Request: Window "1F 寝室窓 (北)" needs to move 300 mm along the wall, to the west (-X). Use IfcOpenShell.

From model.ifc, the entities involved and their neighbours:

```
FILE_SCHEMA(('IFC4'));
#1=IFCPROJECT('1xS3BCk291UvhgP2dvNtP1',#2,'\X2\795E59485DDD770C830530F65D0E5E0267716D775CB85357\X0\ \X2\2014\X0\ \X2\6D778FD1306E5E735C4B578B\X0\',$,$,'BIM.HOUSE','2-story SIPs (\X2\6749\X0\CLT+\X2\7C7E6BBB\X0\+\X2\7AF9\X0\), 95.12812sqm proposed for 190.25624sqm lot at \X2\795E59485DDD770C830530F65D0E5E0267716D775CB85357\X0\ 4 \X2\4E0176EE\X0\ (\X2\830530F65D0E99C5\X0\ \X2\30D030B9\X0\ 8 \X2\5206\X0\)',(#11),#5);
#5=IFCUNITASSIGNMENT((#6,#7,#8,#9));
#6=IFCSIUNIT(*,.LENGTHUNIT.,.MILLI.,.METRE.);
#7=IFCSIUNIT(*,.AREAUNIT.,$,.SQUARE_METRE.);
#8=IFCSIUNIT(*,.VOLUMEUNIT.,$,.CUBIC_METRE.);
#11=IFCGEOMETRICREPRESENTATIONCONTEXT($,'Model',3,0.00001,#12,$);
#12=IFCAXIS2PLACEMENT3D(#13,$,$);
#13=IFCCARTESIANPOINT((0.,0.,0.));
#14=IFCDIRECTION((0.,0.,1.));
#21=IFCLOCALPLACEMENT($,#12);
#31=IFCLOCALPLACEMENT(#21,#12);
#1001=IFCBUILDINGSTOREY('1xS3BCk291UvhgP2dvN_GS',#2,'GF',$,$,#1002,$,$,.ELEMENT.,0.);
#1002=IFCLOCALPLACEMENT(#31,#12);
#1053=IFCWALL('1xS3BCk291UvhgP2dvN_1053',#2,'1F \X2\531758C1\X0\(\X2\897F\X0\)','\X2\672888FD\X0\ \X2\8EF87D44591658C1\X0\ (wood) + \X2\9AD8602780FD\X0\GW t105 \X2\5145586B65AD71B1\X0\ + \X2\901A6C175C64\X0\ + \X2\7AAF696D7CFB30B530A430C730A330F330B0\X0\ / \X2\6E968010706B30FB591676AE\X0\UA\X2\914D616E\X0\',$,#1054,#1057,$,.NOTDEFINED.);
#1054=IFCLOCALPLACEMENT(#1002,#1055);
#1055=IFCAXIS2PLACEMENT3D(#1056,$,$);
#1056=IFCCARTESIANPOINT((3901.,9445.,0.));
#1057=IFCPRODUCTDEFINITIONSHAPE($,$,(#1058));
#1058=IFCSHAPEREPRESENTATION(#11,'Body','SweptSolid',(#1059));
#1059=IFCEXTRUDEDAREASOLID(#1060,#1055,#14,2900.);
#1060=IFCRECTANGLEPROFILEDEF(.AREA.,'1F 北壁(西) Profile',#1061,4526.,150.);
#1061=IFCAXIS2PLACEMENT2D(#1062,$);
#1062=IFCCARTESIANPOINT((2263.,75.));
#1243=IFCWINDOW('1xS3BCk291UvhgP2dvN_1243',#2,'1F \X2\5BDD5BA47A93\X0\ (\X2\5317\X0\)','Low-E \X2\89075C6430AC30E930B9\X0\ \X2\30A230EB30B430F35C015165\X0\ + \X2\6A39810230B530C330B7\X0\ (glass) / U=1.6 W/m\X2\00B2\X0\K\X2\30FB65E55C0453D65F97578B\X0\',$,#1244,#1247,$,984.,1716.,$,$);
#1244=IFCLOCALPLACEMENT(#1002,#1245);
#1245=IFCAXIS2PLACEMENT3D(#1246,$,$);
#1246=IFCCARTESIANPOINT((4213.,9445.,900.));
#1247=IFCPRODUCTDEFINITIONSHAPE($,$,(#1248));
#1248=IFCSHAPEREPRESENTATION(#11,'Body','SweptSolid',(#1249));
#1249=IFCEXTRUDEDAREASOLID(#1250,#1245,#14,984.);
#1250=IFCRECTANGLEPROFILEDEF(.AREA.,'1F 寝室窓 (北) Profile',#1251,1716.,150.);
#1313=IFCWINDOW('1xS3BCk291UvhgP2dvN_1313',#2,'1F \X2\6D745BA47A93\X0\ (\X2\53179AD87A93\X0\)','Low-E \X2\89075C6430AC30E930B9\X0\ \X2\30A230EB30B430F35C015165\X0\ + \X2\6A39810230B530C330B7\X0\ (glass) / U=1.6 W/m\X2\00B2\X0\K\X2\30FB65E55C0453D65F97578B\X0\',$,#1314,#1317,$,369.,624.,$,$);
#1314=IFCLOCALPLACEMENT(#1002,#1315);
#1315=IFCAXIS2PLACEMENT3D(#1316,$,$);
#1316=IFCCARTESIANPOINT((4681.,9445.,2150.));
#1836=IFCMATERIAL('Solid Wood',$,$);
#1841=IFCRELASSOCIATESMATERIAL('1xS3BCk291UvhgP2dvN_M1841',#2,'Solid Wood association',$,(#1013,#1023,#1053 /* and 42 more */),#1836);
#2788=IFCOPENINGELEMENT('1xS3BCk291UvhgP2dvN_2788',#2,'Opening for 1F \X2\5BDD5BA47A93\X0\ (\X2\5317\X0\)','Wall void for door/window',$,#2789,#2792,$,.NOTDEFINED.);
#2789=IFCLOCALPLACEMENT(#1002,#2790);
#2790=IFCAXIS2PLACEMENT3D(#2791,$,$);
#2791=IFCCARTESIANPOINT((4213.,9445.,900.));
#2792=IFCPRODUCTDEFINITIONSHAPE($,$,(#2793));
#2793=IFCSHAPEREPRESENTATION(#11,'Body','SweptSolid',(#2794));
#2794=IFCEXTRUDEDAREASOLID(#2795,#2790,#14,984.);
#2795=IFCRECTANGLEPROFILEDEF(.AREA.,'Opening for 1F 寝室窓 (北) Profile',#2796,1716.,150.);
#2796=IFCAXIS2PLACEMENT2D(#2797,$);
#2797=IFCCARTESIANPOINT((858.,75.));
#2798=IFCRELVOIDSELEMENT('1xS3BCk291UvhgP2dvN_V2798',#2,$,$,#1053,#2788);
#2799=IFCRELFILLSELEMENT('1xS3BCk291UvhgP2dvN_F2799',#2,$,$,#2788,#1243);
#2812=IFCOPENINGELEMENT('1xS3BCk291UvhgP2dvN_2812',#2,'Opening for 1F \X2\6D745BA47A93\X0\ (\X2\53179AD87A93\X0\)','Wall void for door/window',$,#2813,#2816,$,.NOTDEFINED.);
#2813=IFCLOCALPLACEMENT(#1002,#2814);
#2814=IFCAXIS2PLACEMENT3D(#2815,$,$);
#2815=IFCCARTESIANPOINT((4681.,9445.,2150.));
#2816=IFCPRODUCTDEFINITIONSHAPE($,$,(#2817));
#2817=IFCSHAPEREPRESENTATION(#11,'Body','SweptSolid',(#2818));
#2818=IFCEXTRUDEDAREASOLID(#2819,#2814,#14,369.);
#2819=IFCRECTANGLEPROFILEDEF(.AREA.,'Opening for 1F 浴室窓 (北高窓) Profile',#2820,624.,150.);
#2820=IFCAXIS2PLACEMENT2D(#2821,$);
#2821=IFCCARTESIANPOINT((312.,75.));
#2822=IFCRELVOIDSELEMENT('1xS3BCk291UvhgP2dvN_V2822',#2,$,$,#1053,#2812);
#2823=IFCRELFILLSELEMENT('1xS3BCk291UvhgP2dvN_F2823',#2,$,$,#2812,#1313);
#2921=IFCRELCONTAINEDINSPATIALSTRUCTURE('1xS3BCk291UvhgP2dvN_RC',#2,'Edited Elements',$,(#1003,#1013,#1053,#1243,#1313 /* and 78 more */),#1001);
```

```python
import ifcopenshell
import ifcopenshell.api.geometry
import ifcopenshell.util.placement

model = ifcopenshell.open("model.ifc")

window = model.by_guid("1xS3BCk291UvhgP2dvN_1243")
opening = window.FillsVoids[0].RelatingOpeningElement
wall = opening.VoidsElements[0].RelatingBuildingElement

wall_matrix = ifcopenshell.util.placement.get_local_placement(wall.ObjectPlacement)
shift = wall_matrix[:3, 0] * -300.0
before = ifcopenshell.util.placement.get_local_placement(window.ObjectPlacement)[:3, 3].copy()

# The window is not placed relative to its opening, so move both.
for product in (opening, window):
    matrix = ifcopenshell.util.placement.get_local_placement(product.ObjectPlacement)
    matrix[:3, 3] += shift
    ifcopenshell.api.geometry.edit_object_placement(model, product=product, matrix=matrix, is_si=False)

after = ifcopenshell.util.placement.get_local_placement(window.ObjectPlacement)[:3, 3]
print("window moved by", (after - before).round(3) + 0.0)

model.write("model_edited.ifc")
```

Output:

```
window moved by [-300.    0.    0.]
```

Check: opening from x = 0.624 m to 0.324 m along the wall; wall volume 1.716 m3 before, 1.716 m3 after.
